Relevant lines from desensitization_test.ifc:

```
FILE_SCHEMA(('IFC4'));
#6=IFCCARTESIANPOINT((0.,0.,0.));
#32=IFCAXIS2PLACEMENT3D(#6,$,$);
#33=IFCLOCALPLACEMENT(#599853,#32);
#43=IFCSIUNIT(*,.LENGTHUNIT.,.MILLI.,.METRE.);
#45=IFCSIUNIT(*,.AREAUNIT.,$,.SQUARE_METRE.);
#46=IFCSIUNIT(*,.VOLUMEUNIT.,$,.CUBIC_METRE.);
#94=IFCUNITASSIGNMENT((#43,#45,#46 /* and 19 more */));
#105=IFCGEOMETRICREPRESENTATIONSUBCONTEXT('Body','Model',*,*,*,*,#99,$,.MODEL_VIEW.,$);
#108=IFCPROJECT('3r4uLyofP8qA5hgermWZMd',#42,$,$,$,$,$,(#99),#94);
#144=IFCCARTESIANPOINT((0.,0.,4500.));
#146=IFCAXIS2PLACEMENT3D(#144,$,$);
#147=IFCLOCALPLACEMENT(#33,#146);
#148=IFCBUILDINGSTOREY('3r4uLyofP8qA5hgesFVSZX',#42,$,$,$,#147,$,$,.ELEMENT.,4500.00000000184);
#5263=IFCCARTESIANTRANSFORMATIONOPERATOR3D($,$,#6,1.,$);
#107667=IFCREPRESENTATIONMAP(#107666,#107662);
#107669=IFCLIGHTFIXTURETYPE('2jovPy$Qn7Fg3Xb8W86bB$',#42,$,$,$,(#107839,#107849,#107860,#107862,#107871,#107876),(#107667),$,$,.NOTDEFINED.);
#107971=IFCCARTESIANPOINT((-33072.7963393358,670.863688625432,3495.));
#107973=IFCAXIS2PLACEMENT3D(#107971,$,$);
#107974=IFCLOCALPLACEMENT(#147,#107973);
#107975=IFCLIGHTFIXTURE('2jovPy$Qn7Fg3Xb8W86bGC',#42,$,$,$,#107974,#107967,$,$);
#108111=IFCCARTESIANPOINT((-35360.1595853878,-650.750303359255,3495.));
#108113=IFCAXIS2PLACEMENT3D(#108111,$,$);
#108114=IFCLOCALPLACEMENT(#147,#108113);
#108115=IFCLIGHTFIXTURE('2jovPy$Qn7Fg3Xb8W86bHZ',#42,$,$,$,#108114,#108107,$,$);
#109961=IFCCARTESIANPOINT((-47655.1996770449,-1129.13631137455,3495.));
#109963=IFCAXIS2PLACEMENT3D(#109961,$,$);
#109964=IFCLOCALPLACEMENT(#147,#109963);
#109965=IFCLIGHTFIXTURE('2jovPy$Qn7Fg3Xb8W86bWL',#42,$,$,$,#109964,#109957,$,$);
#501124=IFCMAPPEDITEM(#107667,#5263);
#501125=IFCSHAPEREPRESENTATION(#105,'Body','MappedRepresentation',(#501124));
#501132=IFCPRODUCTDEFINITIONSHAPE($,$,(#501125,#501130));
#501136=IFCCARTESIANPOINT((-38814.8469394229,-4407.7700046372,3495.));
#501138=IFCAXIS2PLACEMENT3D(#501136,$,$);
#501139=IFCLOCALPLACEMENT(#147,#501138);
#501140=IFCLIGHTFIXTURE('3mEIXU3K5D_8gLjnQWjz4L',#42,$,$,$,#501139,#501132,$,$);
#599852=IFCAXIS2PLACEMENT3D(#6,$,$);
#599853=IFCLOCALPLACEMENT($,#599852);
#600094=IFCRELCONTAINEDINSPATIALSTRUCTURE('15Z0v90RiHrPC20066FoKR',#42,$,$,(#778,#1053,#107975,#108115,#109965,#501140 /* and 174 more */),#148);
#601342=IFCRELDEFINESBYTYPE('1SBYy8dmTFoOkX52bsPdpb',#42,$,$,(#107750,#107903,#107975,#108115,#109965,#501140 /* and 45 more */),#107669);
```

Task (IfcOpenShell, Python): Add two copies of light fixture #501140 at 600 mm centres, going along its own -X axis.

```python
import ifcopenshell
import ifcopenshell.api.geometry
import ifcopenshell.api.root
import ifcopenshell.util.element
import ifcopenshell.util.placement

model = ifcopenshell.open("desensitization_test.ifc")


def reuse_history(source, copy):
    """copy_class also copies each property set's owner history, people and application; keep the originals."""
    for rel in copy.IsDefinedBy:
        if rel.is_a("IfcRelDefinesByProperties") and (history := rel.RelatingPropertyDefinition.OwnerHistory):
            rel.RelatingPropertyDefinition.OwnerHistory = source.OwnerHistory
            ifcopenshell.util.element.remove_deep2(model, history)


source = model.by_id(501140)
base = ifcopenshell.util.placement.get_local_placement(source.ObjectPlacement)
step = -base[:3, 0] * 600.0

for i in range(1, 3):
    copy = ifcopenshell.api.root.copy_class(model, product=source)
    copy.Representation = ifcopenshell.util.element.copy_deep(
        model, source.Representation, exclude=["IfcGeometricRepresentationContext", "IfcRepresentationMap"]
    )
    reuse_history(source, copy)
    matrix = base.copy()
    matrix[:3, 3] += i * step
    print("added at", matrix[:3, 3].round(3) + 0.0)
    ifcopenshell.api.geometry.edit_object_placement(model, product=copy, matrix=matrix, is_si=False)

model.write("desensitization_test_v2.ifc")
```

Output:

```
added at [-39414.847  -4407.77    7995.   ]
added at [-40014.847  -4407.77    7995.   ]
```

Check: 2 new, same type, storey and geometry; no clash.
